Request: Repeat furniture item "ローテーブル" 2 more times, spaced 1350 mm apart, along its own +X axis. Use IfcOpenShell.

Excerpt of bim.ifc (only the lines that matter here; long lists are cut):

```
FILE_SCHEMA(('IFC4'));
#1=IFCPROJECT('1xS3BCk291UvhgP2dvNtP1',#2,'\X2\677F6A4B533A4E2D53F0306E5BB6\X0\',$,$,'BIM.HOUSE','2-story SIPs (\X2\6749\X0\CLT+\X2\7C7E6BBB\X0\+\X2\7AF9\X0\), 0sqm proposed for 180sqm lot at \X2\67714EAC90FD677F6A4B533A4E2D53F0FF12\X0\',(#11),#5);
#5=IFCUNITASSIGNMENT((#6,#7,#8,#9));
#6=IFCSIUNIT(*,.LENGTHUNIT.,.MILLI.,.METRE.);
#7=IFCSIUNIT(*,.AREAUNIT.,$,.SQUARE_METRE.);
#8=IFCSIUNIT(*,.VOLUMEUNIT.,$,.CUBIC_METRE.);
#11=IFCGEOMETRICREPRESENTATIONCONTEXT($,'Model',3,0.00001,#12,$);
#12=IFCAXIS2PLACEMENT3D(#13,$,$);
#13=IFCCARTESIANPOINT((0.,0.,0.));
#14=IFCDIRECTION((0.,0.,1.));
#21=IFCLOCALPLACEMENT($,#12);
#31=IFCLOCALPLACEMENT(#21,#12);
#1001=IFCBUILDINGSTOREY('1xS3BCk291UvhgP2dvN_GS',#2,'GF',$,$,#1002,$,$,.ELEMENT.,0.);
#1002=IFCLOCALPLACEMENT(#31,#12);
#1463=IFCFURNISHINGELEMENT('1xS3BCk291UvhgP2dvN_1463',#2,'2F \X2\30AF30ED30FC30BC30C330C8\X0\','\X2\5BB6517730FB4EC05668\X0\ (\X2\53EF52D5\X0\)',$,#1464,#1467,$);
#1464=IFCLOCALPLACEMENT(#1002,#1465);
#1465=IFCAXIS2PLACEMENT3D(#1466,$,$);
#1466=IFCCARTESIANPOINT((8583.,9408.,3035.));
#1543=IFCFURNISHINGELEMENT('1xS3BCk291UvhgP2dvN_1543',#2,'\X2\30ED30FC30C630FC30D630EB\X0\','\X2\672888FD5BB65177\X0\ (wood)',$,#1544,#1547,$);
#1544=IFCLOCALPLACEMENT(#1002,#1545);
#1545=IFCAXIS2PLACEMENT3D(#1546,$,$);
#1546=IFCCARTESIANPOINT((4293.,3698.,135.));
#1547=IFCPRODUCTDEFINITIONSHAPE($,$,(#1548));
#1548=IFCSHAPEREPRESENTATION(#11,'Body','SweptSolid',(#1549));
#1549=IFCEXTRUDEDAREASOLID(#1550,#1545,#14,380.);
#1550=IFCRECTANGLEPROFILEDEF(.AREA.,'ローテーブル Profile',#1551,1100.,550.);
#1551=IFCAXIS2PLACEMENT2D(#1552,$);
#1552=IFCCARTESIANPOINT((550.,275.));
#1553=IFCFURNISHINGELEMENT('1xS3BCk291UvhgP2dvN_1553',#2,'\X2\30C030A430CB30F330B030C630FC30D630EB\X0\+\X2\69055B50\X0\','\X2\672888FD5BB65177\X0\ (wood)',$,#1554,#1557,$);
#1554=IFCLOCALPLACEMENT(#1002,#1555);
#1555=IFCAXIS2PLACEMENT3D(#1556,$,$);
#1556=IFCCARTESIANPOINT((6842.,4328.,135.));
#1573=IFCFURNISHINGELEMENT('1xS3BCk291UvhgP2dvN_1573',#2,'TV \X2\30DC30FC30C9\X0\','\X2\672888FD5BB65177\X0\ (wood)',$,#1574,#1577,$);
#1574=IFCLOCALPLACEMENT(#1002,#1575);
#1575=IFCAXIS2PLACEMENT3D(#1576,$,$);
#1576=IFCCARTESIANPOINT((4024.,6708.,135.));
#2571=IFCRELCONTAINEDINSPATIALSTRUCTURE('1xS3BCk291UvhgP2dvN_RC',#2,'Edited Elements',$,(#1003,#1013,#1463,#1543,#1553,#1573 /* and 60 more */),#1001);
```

```python
import ifcopenshell
import ifcopenshell.api.geometry
import ifcopenshell.api.root
import ifcopenshell.util.element
import ifcopenshell.util.placement
import ifcopenshell.util.unit

model = ifcopenshell.open("bim.ifc")
unit_scale = ifcopenshell.util.unit.calculate_unit_scale(model)


def reuse_history(source, copy):
    """copy_class also copies each property set's owner history, people and application; keep the originals."""
    for rel in copy.IsDefinedBy:
        if rel.is_a("IfcRelDefinesByProperties") and (history := rel.RelatingPropertyDefinition.OwnerHistory):
            rel.RelatingPropertyDefinition.OwnerHistory = source.OwnerHistory
            ifcopenshell.util.element.remove_deep2(model, history)


source = model.by_guid("1xS3BCk291UvhgP2dvN_1543")
base = ifcopenshell.util.placement.get_local_placement(source.ObjectPlacement)
step = base[:3, 0] * 1.35 / unit_scale

for i in range(1, 3):
    copy = ifcopenshell.api.root.copy_class(model, product=source)
    copy.Representation = ifcopenshell.util.element.copy_deep(
        model, source.Representation, exclude=["IfcGeometricRepresentationContext", "IfcRepresentationMap"]
    )
    reuse_history(source, copy)
    matrix = base.copy()
    matrix[:3, 3] += i * step
    print("added at", matrix[:3, 3].round(3) + 0.0)
    ifcopenshell.api.geometry.edit_object_placement(model, product=copy, matrix=matrix, is_si=False)

model.write("bim_updated.ifc")
```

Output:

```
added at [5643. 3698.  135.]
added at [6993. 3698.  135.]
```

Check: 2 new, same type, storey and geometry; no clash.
